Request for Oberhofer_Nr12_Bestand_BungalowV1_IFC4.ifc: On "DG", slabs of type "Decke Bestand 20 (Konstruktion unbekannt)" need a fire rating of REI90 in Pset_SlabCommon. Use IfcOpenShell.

First a look at what the model holds.

```python
import ifcopenshell
import ifcopenshell.util.element

model = ifcopenshell.open("Oberhofer_Nr12_Bestand_BungalowV1_IFC4.ifc")
print(model.schema)
storey = next(s for s in model.by_type("IfcBuildingStorey") if s.Name == "DG")
slabs = [e for e in ifcopenshell.util.element.get_decomposition(storey) if e.is_a("IfcSlab")]
seen = {}
for e in slabs:
    element_type = ifcopenshell.util.element.get_type(e)
    key = (element_type.Name if element_type != e and element_type else None, ifcopenshell.util.element.get_pset(e, "Pset_SlabCommon", "FireRating"))
    seen[key] = seen.get(key, 0) + 1
for (name, value), count in sorted(seen.items(), key=str):
    print(count, "x", name, "|", value)
```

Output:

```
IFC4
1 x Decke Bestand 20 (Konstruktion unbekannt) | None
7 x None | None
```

```python
import ifcopenshell
import ifcopenshell.api.pset
import ifcopenshell.util.element

model = ifcopenshell.open("Oberhofer_Nr12_Bestand_BungalowV1_IFC4.ifc")

storey = next(s for s in model.by_type("IfcBuildingStorey") if s.Name == "DG")
slabs = [e for e in ifcopenshell.util.element.get_decomposition(storey) if e.is_a("IfcSlab")]

count = 0
for e in slabs:
    element_type = ifcopenshell.util.element.get_type(e)
    if element_type in (None, e) or element_type.Name != "Decke Bestand 20 (Konstruktion unbekannt)":
        continue
    # add_pset returns the element's existing set when there is one.
    pset = ifcopenshell.api.pset.add_pset(model, product=e, name="Pset_SlabCommon")
    ifcopenshell.api.pset.edit_pset(model, pset=pset, properties={"FireRating": "REI90"})
    count += 1

print(count, "slabs updated")

model.write("Oberhofer_Nr12_Bestand_BungalowV1_IFC4_v2.ifc")
```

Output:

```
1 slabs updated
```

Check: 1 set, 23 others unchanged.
